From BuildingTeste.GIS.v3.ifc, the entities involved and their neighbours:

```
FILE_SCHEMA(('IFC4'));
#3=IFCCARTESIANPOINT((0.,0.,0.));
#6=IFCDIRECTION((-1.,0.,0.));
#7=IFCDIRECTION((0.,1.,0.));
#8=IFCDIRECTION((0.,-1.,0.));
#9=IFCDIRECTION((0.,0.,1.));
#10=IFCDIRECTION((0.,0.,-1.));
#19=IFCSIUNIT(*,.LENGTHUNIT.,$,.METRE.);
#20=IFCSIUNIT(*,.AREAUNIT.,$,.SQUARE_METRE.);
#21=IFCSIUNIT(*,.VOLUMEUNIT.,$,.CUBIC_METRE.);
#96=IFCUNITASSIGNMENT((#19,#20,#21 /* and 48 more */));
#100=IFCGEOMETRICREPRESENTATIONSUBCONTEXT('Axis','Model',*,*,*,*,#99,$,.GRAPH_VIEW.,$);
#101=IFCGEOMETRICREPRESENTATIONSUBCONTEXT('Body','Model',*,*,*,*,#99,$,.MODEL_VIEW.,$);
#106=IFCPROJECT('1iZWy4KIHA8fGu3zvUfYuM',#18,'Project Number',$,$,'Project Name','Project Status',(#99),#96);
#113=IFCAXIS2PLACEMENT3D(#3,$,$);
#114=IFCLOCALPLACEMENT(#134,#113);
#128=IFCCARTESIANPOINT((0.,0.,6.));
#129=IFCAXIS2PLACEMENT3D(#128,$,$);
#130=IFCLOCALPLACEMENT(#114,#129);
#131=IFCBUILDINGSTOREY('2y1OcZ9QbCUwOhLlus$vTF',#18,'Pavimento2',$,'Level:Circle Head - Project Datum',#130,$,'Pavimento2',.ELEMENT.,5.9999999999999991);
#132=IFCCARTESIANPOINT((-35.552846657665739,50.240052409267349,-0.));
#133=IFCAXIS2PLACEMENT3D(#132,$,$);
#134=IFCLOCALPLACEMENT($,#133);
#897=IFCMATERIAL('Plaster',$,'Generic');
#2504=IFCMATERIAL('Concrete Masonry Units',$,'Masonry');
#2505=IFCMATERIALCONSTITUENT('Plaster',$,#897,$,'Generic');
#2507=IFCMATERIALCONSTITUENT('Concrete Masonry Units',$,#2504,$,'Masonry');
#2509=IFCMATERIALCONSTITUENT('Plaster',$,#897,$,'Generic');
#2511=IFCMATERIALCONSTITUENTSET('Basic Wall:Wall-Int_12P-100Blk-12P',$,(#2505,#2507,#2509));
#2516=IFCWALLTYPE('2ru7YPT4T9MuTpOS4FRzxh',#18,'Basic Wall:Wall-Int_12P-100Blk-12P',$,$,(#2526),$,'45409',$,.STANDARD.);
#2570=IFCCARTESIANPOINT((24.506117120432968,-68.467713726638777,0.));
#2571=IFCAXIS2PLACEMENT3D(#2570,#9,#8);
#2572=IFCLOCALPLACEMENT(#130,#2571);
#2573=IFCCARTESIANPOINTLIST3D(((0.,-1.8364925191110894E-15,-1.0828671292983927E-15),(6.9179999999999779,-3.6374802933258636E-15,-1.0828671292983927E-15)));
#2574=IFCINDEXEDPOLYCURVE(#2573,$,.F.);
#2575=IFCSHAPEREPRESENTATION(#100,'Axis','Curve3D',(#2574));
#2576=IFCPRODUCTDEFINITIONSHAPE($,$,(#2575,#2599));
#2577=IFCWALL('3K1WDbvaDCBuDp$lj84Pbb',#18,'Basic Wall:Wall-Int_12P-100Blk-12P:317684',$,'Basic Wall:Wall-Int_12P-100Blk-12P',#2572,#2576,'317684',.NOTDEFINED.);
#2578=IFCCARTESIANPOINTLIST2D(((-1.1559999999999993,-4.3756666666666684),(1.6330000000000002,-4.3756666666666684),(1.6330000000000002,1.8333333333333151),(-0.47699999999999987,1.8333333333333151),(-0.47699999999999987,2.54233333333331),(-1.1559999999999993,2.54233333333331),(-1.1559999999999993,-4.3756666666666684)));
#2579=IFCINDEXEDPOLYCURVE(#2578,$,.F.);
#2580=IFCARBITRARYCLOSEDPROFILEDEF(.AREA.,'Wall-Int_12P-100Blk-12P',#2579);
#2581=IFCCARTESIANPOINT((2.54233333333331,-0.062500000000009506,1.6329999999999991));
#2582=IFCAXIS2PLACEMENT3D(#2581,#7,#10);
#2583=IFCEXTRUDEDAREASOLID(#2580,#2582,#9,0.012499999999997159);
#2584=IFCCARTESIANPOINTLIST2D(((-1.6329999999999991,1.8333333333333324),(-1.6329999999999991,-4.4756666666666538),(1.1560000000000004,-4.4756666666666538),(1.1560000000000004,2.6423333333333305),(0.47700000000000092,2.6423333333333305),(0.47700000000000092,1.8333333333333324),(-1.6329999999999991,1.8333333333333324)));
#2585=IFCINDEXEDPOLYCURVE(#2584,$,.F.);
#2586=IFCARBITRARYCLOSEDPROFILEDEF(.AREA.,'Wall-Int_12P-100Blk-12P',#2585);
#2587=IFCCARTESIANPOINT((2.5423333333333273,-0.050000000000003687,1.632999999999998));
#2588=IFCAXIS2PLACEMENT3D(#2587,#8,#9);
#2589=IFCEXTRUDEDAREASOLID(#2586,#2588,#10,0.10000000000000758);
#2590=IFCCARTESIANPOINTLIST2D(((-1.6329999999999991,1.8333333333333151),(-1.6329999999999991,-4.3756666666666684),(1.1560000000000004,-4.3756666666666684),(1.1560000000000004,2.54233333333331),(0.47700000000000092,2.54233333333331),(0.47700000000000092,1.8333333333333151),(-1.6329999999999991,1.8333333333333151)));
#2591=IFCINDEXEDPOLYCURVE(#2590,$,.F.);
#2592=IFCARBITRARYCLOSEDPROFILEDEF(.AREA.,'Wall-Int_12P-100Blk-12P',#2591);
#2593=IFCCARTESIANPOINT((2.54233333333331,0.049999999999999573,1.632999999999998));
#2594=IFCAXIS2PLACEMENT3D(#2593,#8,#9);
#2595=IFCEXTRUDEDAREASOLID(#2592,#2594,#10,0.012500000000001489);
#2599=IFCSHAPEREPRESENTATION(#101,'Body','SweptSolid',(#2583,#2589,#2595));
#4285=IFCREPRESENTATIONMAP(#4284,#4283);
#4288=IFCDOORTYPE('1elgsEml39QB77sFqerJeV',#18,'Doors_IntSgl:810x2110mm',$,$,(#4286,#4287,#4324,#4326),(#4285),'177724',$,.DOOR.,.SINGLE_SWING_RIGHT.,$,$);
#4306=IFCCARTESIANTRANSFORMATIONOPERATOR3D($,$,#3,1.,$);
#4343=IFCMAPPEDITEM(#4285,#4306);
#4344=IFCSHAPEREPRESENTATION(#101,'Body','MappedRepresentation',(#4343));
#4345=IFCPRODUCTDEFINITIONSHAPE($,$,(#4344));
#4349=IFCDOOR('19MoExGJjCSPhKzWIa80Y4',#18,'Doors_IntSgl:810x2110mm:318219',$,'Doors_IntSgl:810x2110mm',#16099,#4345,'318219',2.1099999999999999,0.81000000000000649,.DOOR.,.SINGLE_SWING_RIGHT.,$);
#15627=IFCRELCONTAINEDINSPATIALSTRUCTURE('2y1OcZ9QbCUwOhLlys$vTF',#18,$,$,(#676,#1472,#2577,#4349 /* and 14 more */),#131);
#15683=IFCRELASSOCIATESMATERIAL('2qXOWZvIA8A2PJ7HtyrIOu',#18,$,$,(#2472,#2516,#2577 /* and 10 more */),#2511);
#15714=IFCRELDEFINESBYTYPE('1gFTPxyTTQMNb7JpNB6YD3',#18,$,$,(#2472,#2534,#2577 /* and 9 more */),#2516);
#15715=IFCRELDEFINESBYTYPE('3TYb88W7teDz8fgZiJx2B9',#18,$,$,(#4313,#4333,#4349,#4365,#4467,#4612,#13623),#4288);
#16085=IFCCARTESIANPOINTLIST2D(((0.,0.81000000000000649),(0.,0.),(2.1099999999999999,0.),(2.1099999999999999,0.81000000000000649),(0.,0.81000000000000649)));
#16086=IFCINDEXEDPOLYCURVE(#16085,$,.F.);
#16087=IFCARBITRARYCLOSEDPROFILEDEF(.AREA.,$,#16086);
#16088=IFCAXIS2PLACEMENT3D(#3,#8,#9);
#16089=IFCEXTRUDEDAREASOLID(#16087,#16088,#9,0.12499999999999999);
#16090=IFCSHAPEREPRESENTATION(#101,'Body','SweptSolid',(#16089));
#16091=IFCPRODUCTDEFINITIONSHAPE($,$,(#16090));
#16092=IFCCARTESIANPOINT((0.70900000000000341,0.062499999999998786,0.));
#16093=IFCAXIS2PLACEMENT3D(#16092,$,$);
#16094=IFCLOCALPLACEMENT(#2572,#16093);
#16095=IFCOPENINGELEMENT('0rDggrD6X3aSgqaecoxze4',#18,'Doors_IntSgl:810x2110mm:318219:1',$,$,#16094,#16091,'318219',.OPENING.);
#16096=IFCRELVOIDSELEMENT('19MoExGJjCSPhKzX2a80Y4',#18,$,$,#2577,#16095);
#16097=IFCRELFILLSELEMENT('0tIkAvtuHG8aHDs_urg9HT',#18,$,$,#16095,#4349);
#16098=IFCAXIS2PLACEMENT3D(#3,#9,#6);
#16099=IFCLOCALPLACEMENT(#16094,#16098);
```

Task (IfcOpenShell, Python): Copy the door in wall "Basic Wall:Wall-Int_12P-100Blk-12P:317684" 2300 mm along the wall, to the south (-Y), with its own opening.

```python
import ifcopenshell
import ifcopenshell.api.feature
import ifcopenshell.api.geometry
import ifcopenshell.api.root
import ifcopenshell.geom
import ifcopenshell.util.element
import ifcopenshell.util.placement
import ifcopenshell.util.shape
import ifcopenshell.util.unit

model = ifcopenshell.open("BuildingTeste.GIS.v3.ifc")
unit_scale = ifcopenshell.util.unit.calculate_unit_scale(model)
settings = ifcopenshell.geom.settings()


def volume(element):
    """Net volume in cubic metres, openings subtracted."""
    shape = ifcopenshell.geom.create_shape(settings, element)
    return ifcopenshell.util.shape.get_volume(shape.geometry)


def reuse_history(source, copy):
    """copy_class also copies each property set's owner history, people and application; keep the originals."""
    for rel in copy.IsDefinedBy:
        if rel.is_a("IfcRelDefinesByProperties") and (history := rel.RelatingPropertyDefinition.OwnerHistory):
            rel.RelatingPropertyDefinition.OwnerHistory = source.OwnerHistory
            ifcopenshell.util.element.remove_deep2(model, history)


door = model.by_guid("19MoExGJjCSPhKzWIa80Y4")
opening = door.FillsVoids[0].RelatingOpeningElement
wall = opening.VoidsElements[0].RelatingBuildingElement
before = volume(wall)
shift = ifcopenshell.util.placement.get_local_placement(wall.ObjectPlacement)[:3, 0] * 2.3 / unit_scale

# copy_class copies the void relationship, type, container and properties, but no geometry.
new_opening = ifcopenshell.api.root.copy_class(model, product=opening)
new_opening.Representation = ifcopenshell.util.element.copy_deep(
    model, opening.Representation, exclude=["IfcGeometricRepresentationContext", "IfcRepresentationMap"]
)
new_opening.Name = "Doors_IntSgl:810x2110mm"
new_opening.Tag = None
new_door = ifcopenshell.api.root.copy_class(model, product=door)
new_door.Representation = ifcopenshell.util.element.copy_deep(
    model, door.Representation, exclude=["IfcGeometricRepresentationContext", "IfcRepresentationMap"]
)
new_door.Name = "Doors_IntSgl:810x2110mm"
new_door.Tag = None
reuse_history(door, new_door)
ifcopenshell.api.feature.add_filling(model, opening=new_opening, element=new_door)

for old, new in ((opening, new_opening), (door, new_door)):
    matrix = ifcopenshell.util.placement.get_local_placement(old.ObjectPlacement)
    matrix[:3, 3] += shift
    ifcopenshell.api.geometry.edit_object_placement(model, product=new, matrix=matrix, is_si=False)

after = volume(wall)

print(f"wall volume {before:.3f} -> {after:.3f} m3")

model.write("BuildingTeste.GIS.v3-out.ifc")
```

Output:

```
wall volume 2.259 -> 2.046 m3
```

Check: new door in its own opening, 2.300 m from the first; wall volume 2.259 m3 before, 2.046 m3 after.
